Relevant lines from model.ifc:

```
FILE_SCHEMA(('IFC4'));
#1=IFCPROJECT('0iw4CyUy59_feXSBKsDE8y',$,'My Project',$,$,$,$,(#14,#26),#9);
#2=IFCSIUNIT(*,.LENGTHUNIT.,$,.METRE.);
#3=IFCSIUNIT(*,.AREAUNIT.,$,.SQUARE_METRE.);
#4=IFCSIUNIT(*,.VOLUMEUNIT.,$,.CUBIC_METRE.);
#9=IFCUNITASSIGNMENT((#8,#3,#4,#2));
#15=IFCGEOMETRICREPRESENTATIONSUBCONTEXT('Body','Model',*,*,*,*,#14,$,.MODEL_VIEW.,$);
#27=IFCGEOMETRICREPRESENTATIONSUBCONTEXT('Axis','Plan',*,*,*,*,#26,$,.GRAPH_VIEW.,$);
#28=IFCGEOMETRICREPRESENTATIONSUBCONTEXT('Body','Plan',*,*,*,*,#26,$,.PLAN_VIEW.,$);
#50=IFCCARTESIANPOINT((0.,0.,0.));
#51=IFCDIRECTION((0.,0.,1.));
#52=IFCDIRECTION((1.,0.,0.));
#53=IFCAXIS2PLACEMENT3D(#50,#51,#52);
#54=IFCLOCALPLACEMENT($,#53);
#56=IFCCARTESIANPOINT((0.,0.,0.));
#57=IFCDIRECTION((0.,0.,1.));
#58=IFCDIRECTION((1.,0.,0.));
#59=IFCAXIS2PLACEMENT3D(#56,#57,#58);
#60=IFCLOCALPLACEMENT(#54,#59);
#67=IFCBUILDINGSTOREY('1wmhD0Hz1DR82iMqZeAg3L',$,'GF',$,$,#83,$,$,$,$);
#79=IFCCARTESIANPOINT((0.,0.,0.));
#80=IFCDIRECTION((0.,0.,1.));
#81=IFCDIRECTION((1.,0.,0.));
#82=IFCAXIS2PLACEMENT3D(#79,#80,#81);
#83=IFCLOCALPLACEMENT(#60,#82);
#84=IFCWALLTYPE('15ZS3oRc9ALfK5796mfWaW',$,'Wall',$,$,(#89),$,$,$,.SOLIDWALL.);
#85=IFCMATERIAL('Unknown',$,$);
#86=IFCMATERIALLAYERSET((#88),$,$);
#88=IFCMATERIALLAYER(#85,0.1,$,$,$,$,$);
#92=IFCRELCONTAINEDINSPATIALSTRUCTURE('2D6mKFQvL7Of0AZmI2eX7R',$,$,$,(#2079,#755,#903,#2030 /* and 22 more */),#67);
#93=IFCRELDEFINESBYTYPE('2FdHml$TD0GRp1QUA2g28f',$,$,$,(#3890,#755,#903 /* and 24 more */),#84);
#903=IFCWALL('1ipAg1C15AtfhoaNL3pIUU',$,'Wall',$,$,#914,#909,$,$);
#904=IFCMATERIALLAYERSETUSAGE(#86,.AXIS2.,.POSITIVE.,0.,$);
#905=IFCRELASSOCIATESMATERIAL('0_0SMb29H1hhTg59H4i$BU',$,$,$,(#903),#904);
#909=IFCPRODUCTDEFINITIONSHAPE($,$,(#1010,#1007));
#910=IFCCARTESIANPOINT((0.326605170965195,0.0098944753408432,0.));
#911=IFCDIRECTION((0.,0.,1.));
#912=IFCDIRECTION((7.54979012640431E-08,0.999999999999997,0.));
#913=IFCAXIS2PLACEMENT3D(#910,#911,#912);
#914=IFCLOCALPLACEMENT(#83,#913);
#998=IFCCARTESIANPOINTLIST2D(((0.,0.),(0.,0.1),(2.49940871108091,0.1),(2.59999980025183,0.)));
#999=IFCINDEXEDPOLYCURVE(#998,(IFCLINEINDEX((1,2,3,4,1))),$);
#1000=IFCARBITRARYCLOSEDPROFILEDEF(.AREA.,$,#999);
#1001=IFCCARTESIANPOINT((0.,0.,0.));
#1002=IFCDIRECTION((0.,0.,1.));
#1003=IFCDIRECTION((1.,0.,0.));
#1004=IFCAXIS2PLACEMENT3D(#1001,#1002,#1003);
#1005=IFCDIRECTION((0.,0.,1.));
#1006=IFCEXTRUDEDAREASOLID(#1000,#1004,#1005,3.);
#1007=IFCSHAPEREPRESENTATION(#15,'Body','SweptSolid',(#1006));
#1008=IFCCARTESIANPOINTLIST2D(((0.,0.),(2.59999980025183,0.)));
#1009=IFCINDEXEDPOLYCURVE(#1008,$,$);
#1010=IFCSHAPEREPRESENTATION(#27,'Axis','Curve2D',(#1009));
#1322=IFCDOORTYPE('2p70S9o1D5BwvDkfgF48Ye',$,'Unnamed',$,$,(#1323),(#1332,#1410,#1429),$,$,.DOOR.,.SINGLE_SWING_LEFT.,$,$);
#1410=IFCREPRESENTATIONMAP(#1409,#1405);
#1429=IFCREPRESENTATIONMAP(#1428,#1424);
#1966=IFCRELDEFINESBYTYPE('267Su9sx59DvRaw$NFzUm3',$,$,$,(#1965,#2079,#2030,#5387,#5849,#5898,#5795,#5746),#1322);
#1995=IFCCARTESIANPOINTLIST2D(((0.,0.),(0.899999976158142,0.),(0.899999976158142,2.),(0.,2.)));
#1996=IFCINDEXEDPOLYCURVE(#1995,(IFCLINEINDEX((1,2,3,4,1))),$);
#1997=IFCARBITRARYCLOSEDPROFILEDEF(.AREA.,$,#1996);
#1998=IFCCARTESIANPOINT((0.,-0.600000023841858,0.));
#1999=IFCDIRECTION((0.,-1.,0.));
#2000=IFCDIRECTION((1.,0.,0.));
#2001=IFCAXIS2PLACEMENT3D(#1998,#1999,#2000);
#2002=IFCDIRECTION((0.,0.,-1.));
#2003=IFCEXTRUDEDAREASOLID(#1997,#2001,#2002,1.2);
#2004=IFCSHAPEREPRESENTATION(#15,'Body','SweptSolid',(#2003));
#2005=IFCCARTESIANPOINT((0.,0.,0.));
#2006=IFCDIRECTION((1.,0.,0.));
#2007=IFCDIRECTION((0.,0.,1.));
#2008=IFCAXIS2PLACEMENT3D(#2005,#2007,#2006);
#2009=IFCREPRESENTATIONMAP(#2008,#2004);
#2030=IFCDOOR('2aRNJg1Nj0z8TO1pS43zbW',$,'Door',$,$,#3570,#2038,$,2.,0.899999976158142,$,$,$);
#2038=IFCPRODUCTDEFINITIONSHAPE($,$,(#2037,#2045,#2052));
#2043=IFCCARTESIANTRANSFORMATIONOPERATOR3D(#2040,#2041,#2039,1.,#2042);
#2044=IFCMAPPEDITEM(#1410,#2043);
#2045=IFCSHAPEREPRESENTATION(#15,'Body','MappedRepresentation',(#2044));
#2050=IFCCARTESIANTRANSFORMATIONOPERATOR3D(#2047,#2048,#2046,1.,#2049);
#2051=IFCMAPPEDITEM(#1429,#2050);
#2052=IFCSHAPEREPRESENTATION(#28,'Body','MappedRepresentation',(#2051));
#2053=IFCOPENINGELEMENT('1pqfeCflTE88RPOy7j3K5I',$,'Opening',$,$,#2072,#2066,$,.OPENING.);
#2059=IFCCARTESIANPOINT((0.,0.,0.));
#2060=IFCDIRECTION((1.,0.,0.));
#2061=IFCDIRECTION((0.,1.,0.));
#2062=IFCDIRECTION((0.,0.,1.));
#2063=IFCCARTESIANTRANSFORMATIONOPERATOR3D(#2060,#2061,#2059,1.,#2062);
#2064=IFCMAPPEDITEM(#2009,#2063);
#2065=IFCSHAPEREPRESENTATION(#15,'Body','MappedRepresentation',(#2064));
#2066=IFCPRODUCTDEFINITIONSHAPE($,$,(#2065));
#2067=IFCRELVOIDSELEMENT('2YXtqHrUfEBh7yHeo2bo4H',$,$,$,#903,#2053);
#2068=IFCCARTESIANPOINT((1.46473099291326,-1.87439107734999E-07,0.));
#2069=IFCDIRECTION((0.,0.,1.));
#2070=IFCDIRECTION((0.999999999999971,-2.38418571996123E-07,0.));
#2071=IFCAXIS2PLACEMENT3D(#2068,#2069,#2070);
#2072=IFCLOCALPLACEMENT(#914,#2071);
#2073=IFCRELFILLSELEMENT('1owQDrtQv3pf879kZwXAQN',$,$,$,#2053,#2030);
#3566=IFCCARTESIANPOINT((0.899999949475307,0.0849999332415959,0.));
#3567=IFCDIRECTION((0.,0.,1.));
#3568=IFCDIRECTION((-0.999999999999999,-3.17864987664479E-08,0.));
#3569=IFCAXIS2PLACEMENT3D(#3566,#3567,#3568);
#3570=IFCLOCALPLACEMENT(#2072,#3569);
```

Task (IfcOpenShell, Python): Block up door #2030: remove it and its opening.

```python
import ifcopenshell
import ifcopenshell.api.feature
import ifcopenshell.api.root
import ifcopenshell.geom
import ifcopenshell.util.shape

model = ifcopenshell.open("model.ifc")
settings = ifcopenshell.geom.settings()


def volume(element):
    """Net volume in cubic metres, openings subtracted."""
    shape = ifcopenshell.geom.create_shape(settings, element)
    return ifcopenshell.util.shape.get_volume(shape.geometry)


door = model.by_guid("2aRNJg1Nj0z8TO1pS43zbW")
opening = door.FillsVoids[0].RelatingOpeningElement
wall = opening.VoidsElements[0].RelatingBuildingElement
before = volume(wall)

ifcopenshell.api.root.remove_product(model, product=door)
ifcopenshell.api.feature.remove_feature(model, feature=opening)

after = volume(wall)

print(f"wall volume {before:.3f} -> {after:.3f} m3")

model.write("model-out.ifc")
```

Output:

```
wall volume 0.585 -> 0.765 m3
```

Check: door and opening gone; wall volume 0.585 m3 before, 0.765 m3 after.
